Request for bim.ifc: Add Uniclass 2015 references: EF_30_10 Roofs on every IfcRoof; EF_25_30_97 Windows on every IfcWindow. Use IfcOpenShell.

First a look at what the model holds.

```python
import ifcopenshell

model = ifcopenshell.open("bim.ifc")
print(model.schema)
print("classifications:", [c.Name for c in model.by_type("IfcClassification")])
for ifc_class in ("IfcDoor", "IfcRoof", "IfcStair", "IfcWall", "IfcWindow"):
    print(ifc_class, len(model.by_type(ifc_class)))
```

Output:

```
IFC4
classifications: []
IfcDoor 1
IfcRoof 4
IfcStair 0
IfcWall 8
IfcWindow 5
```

```python
import ifcopenshell
import ifcopenshell.api.classification

model = ifcopenshell.open("bim.ifc")

system = ifcopenshell.api.classification.add_classification(model, classification="Uniclass 2015")

codes = {
    "IfcRoof": ("EF_30_10", "Roofs"),
    "IfcWindow": ("EF_25_30_97", "Windows"),
}
for ifc_class, (code, name) in codes.items():
    products = model.by_type(ifc_class)
    ifcopenshell.api.classification.add_reference(
        model, products=products, classification=system, identification=code, name=name
    )
    print(code, len(products))

model.write("bim_rev.ifc")
```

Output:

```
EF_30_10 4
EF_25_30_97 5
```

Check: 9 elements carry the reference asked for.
